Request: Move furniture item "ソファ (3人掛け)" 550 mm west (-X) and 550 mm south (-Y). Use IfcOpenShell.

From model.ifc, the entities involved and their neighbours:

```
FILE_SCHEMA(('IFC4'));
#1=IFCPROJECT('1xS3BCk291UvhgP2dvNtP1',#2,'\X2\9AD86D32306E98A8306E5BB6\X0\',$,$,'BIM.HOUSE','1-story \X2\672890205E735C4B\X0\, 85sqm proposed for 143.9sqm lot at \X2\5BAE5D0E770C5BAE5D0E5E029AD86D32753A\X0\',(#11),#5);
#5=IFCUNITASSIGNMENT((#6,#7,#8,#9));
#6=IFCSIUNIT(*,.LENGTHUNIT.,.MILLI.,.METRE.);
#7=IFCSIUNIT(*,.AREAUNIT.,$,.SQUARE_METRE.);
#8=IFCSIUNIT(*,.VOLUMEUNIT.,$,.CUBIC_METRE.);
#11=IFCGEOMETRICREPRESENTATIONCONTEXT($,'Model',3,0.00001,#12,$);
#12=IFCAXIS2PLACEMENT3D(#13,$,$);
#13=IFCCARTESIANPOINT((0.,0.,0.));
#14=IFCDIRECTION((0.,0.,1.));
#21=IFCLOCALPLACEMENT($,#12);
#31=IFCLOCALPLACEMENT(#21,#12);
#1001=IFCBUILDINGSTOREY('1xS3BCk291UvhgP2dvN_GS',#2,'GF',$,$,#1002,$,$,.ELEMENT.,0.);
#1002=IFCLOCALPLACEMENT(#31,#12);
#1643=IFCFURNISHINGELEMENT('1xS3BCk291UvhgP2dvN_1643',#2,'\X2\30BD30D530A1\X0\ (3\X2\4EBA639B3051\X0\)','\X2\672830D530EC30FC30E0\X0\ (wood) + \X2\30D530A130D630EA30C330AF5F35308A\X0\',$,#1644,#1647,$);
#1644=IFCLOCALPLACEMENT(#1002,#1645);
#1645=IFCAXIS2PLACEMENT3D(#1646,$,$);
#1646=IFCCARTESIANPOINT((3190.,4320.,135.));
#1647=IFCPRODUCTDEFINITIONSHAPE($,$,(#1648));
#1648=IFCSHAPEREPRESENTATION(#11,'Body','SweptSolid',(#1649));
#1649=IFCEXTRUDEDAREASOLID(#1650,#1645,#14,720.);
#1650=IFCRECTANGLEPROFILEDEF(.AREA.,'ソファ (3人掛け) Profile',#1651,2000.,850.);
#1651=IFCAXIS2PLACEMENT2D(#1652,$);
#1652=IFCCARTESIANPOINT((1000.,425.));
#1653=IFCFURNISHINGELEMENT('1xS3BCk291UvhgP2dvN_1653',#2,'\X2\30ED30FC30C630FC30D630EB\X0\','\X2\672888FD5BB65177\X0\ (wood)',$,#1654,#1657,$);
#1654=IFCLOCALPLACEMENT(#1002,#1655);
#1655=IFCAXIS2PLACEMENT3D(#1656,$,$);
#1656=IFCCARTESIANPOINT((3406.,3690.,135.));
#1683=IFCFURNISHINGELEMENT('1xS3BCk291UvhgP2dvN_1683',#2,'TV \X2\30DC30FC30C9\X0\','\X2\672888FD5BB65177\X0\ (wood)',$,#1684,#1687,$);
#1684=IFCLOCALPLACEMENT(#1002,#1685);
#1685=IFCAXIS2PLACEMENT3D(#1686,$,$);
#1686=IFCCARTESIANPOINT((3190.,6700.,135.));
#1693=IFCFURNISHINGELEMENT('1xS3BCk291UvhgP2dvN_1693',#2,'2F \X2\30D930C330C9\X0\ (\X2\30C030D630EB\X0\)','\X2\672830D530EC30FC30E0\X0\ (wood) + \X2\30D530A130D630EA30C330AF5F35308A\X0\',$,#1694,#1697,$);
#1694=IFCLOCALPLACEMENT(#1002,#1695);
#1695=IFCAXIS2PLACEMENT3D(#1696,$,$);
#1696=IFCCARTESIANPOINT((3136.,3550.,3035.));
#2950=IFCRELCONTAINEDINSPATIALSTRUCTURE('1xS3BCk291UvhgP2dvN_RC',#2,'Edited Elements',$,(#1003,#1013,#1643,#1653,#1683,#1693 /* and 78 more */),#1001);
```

```python
import ifcopenshell
import ifcopenshell.api.geometry
import ifcopenshell.util.placement
import ifcopenshell.util.unit

model = ifcopenshell.open("model.ifc")
unit_scale = ifcopenshell.util.unit.calculate_unit_scale(model)

item = model.by_guid("1xS3BCk291UvhgP2dvN_1643")
matrix = ifcopenshell.util.placement.get_local_placement(item.ObjectPlacement)
matrix[0, 3] -= 0.55 / unit_scale
matrix[1, 3] -= 0.55 / unit_scale
ifcopenshell.api.geometry.edit_object_placement(model, product=item, matrix=matrix, is_si=False)

print(ifcopenshell.util.placement.get_local_placement(item.ObjectPlacement).round(3) + 0.0)

model.write("model-out.ifc")
```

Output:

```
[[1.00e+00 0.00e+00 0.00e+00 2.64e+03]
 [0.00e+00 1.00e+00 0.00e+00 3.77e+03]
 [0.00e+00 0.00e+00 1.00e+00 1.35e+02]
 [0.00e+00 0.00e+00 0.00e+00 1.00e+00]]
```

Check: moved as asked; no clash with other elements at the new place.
